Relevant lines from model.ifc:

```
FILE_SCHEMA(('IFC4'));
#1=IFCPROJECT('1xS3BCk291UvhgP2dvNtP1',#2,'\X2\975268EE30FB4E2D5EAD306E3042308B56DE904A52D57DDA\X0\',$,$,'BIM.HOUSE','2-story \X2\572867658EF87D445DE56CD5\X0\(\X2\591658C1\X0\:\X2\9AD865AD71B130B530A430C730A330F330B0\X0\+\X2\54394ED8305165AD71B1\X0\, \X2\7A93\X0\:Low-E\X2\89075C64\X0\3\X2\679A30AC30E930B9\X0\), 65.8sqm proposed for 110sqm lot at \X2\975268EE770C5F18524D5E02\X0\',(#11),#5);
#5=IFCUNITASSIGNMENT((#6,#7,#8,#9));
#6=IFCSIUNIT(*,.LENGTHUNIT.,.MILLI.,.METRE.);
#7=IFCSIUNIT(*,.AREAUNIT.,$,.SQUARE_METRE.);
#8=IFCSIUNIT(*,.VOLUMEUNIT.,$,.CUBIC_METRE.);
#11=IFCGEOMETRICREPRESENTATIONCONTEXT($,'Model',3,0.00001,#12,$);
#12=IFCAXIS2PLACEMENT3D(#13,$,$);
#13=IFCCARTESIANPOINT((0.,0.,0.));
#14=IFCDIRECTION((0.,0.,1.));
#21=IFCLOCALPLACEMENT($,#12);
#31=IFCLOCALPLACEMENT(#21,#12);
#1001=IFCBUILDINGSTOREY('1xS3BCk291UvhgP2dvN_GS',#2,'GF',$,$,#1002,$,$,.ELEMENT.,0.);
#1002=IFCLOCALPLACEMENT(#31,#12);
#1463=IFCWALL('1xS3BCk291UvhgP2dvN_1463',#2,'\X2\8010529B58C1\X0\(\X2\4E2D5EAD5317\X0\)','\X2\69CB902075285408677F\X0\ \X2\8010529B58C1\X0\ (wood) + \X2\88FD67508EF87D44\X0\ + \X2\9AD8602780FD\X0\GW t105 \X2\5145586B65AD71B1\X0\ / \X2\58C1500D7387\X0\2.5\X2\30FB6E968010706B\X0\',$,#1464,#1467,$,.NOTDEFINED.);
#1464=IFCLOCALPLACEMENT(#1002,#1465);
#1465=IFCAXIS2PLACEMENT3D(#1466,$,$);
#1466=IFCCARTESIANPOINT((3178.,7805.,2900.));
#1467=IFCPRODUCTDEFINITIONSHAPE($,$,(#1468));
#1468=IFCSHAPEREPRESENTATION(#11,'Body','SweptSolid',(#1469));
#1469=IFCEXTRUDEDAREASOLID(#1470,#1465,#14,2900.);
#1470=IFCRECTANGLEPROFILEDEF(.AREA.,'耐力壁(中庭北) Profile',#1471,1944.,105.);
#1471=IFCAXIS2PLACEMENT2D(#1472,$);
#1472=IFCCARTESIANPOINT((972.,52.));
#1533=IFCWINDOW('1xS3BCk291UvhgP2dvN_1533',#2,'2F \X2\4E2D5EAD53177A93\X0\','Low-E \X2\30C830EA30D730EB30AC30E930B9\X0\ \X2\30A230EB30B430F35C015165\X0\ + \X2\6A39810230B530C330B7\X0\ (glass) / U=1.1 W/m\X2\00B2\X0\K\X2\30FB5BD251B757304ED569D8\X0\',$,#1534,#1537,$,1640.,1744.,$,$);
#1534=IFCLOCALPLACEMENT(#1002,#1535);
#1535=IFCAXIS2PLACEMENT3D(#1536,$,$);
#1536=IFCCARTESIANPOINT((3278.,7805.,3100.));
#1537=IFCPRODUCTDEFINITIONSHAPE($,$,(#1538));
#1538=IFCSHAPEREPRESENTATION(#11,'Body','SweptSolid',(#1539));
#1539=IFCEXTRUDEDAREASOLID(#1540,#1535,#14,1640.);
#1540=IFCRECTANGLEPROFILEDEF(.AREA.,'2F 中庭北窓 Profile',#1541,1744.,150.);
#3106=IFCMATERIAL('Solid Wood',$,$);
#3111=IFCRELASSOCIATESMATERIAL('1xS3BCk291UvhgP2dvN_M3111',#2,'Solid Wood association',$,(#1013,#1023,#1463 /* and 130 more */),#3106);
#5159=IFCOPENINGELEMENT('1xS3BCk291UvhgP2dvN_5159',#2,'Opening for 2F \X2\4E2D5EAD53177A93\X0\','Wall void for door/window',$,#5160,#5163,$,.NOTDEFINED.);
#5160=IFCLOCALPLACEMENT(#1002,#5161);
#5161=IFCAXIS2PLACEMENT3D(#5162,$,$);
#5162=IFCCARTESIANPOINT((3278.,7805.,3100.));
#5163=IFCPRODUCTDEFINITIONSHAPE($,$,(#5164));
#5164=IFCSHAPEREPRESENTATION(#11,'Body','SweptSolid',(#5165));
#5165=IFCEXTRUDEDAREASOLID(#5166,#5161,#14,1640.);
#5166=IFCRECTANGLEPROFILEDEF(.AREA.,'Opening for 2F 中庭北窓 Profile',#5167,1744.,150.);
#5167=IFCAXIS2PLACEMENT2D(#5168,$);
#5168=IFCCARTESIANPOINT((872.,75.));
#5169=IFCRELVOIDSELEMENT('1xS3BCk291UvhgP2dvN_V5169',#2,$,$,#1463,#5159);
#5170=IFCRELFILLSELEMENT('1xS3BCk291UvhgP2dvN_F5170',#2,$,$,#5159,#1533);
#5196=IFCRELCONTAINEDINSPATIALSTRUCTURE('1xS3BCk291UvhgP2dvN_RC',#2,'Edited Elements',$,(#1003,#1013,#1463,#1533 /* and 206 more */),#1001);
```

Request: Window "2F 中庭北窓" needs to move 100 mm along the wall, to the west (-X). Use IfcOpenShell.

```python
import ifcopenshell
import ifcopenshell.api.geometry
import ifcopenshell.util.placement
import ifcopenshell.util.unit

model = ifcopenshell.open("model.ifc")
unit_scale = ifcopenshell.util.unit.calculate_unit_scale(model)

window = model.by_id(1533)
opening = window.FillsVoids[0].RelatingOpeningElement
wall = opening.VoidsElements[0].RelatingBuildingElement

wall_matrix = ifcopenshell.util.placement.get_local_placement(wall.ObjectPlacement)
shift = wall_matrix[:3, 0] * -0.1 / unit_scale
before = ifcopenshell.util.placement.get_local_placement(window.ObjectPlacement)[:3, 3].copy()

# The window is not placed relative to its opening, so move both.
for product in (opening, window):
    matrix = ifcopenshell.util.placement.get_local_placement(product.ObjectPlacement)
    matrix[:3, 3] += shift
    ifcopenshell.api.geometry.edit_object_placement(model, product=product, matrix=matrix, is_si=False)

after = ifcopenshell.util.placement.get_local_placement(window.ObjectPlacement)[:3, 3]
print("window moved by", (after - before).round(3) + 0.0)

model.write("model_edited.ifc")
```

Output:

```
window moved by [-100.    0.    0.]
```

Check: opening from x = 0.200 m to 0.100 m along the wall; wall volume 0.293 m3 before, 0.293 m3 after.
